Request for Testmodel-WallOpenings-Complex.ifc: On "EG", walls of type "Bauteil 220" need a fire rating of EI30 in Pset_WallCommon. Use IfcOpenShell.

First a look at what the model holds.

```python
import ifcopenshell
import ifcopenshell.util.element

model = ifcopenshell.open("Testmodel-WallOpenings-Complex.ifc")
print(model.schema)
storey = next(s for s in model.by_type("IfcBuildingStorey") if s.Name == "EG")
walls = [e for e in ifcopenshell.util.element.get_decomposition(storey) if e.is_a("IfcWall")]
seen = {}
for e in walls:
    element_type = ifcopenshell.util.element.get_type(e)
    key = (element_type.Name if element_type != e and element_type else None, ifcopenshell.util.element.get_pset(e, "Pset_WallCommon", "FireRating"))
    seen[key] = seen.get(key, 0) + 1
for (name, value), count in sorted(seen.items(), key=str):
    print(count, "x", name, "|", value)
```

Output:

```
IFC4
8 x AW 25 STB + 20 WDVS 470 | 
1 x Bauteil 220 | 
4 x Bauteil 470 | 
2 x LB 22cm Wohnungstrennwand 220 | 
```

```python
import ifcopenshell
import ifcopenshell.api.pset
import ifcopenshell.util.element

model = ifcopenshell.open("Testmodel-WallOpenings-Complex.ifc")

storey = next(s for s in model.by_type("IfcBuildingStorey") if s.Name == "EG")
walls = [e for e in ifcopenshell.util.element.get_decomposition(storey) if e.is_a("IfcWall")]

count = 0
for e in walls:
    element_type = ifcopenshell.util.element.get_type(e)
    if element_type in (None, e) or element_type.Name != "Bauteil 220":
        continue
    # add_pset returns the element's existing set when there is one.
    pset = ifcopenshell.api.pset.add_pset(model, product=e, name="Pset_WallCommon")
    ifcopenshell.api.pset.edit_pset(model, pset=pset, properties={"FireRating": "EI30"})
    count += 1

print(count, "walls updated")

model.write("Testmodel-WallOpenings-Complex_updated.ifc")
```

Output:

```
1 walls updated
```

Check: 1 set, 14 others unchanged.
